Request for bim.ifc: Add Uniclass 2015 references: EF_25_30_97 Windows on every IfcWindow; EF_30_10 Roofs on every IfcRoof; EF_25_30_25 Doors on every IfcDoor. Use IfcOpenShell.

First a look at what the model holds.

```python
import ifcopenshell

model = ifcopenshell.open("bim.ifc")
print(model.schema)
print("classifications:", [c.Name for c in model.by_type("IfcClassification")])
for ifc_class in ("IfcDoor", "IfcRoof", "IfcStair", "IfcWall", "IfcWindow"):
    print(ifc_class, len(model.by_type(ifc_class)))
```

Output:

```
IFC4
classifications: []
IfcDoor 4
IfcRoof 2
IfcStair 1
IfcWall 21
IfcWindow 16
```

```python
import ifcopenshell
import ifcopenshell.api.classification

model = ifcopenshell.open("bim.ifc")

system = ifcopenshell.api.classification.add_classification(model, classification="Uniclass 2015")

codes = {
    "IfcWindow": ("EF_25_30_97", "Windows"),
    "IfcRoof": ("EF_30_10", "Roofs"),
    "IfcDoor": ("EF_25_30_25", "Doors"),
}
for ifc_class, (code, name) in codes.items():
    products = model.by_type(ifc_class)
    ifcopenshell.api.classification.add_reference(
        model, products=products, classification=system, identification=code, name=name
    )
    print(code, len(products))

model.write("bim_edited.ifc")
```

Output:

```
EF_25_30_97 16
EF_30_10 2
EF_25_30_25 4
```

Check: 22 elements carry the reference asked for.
